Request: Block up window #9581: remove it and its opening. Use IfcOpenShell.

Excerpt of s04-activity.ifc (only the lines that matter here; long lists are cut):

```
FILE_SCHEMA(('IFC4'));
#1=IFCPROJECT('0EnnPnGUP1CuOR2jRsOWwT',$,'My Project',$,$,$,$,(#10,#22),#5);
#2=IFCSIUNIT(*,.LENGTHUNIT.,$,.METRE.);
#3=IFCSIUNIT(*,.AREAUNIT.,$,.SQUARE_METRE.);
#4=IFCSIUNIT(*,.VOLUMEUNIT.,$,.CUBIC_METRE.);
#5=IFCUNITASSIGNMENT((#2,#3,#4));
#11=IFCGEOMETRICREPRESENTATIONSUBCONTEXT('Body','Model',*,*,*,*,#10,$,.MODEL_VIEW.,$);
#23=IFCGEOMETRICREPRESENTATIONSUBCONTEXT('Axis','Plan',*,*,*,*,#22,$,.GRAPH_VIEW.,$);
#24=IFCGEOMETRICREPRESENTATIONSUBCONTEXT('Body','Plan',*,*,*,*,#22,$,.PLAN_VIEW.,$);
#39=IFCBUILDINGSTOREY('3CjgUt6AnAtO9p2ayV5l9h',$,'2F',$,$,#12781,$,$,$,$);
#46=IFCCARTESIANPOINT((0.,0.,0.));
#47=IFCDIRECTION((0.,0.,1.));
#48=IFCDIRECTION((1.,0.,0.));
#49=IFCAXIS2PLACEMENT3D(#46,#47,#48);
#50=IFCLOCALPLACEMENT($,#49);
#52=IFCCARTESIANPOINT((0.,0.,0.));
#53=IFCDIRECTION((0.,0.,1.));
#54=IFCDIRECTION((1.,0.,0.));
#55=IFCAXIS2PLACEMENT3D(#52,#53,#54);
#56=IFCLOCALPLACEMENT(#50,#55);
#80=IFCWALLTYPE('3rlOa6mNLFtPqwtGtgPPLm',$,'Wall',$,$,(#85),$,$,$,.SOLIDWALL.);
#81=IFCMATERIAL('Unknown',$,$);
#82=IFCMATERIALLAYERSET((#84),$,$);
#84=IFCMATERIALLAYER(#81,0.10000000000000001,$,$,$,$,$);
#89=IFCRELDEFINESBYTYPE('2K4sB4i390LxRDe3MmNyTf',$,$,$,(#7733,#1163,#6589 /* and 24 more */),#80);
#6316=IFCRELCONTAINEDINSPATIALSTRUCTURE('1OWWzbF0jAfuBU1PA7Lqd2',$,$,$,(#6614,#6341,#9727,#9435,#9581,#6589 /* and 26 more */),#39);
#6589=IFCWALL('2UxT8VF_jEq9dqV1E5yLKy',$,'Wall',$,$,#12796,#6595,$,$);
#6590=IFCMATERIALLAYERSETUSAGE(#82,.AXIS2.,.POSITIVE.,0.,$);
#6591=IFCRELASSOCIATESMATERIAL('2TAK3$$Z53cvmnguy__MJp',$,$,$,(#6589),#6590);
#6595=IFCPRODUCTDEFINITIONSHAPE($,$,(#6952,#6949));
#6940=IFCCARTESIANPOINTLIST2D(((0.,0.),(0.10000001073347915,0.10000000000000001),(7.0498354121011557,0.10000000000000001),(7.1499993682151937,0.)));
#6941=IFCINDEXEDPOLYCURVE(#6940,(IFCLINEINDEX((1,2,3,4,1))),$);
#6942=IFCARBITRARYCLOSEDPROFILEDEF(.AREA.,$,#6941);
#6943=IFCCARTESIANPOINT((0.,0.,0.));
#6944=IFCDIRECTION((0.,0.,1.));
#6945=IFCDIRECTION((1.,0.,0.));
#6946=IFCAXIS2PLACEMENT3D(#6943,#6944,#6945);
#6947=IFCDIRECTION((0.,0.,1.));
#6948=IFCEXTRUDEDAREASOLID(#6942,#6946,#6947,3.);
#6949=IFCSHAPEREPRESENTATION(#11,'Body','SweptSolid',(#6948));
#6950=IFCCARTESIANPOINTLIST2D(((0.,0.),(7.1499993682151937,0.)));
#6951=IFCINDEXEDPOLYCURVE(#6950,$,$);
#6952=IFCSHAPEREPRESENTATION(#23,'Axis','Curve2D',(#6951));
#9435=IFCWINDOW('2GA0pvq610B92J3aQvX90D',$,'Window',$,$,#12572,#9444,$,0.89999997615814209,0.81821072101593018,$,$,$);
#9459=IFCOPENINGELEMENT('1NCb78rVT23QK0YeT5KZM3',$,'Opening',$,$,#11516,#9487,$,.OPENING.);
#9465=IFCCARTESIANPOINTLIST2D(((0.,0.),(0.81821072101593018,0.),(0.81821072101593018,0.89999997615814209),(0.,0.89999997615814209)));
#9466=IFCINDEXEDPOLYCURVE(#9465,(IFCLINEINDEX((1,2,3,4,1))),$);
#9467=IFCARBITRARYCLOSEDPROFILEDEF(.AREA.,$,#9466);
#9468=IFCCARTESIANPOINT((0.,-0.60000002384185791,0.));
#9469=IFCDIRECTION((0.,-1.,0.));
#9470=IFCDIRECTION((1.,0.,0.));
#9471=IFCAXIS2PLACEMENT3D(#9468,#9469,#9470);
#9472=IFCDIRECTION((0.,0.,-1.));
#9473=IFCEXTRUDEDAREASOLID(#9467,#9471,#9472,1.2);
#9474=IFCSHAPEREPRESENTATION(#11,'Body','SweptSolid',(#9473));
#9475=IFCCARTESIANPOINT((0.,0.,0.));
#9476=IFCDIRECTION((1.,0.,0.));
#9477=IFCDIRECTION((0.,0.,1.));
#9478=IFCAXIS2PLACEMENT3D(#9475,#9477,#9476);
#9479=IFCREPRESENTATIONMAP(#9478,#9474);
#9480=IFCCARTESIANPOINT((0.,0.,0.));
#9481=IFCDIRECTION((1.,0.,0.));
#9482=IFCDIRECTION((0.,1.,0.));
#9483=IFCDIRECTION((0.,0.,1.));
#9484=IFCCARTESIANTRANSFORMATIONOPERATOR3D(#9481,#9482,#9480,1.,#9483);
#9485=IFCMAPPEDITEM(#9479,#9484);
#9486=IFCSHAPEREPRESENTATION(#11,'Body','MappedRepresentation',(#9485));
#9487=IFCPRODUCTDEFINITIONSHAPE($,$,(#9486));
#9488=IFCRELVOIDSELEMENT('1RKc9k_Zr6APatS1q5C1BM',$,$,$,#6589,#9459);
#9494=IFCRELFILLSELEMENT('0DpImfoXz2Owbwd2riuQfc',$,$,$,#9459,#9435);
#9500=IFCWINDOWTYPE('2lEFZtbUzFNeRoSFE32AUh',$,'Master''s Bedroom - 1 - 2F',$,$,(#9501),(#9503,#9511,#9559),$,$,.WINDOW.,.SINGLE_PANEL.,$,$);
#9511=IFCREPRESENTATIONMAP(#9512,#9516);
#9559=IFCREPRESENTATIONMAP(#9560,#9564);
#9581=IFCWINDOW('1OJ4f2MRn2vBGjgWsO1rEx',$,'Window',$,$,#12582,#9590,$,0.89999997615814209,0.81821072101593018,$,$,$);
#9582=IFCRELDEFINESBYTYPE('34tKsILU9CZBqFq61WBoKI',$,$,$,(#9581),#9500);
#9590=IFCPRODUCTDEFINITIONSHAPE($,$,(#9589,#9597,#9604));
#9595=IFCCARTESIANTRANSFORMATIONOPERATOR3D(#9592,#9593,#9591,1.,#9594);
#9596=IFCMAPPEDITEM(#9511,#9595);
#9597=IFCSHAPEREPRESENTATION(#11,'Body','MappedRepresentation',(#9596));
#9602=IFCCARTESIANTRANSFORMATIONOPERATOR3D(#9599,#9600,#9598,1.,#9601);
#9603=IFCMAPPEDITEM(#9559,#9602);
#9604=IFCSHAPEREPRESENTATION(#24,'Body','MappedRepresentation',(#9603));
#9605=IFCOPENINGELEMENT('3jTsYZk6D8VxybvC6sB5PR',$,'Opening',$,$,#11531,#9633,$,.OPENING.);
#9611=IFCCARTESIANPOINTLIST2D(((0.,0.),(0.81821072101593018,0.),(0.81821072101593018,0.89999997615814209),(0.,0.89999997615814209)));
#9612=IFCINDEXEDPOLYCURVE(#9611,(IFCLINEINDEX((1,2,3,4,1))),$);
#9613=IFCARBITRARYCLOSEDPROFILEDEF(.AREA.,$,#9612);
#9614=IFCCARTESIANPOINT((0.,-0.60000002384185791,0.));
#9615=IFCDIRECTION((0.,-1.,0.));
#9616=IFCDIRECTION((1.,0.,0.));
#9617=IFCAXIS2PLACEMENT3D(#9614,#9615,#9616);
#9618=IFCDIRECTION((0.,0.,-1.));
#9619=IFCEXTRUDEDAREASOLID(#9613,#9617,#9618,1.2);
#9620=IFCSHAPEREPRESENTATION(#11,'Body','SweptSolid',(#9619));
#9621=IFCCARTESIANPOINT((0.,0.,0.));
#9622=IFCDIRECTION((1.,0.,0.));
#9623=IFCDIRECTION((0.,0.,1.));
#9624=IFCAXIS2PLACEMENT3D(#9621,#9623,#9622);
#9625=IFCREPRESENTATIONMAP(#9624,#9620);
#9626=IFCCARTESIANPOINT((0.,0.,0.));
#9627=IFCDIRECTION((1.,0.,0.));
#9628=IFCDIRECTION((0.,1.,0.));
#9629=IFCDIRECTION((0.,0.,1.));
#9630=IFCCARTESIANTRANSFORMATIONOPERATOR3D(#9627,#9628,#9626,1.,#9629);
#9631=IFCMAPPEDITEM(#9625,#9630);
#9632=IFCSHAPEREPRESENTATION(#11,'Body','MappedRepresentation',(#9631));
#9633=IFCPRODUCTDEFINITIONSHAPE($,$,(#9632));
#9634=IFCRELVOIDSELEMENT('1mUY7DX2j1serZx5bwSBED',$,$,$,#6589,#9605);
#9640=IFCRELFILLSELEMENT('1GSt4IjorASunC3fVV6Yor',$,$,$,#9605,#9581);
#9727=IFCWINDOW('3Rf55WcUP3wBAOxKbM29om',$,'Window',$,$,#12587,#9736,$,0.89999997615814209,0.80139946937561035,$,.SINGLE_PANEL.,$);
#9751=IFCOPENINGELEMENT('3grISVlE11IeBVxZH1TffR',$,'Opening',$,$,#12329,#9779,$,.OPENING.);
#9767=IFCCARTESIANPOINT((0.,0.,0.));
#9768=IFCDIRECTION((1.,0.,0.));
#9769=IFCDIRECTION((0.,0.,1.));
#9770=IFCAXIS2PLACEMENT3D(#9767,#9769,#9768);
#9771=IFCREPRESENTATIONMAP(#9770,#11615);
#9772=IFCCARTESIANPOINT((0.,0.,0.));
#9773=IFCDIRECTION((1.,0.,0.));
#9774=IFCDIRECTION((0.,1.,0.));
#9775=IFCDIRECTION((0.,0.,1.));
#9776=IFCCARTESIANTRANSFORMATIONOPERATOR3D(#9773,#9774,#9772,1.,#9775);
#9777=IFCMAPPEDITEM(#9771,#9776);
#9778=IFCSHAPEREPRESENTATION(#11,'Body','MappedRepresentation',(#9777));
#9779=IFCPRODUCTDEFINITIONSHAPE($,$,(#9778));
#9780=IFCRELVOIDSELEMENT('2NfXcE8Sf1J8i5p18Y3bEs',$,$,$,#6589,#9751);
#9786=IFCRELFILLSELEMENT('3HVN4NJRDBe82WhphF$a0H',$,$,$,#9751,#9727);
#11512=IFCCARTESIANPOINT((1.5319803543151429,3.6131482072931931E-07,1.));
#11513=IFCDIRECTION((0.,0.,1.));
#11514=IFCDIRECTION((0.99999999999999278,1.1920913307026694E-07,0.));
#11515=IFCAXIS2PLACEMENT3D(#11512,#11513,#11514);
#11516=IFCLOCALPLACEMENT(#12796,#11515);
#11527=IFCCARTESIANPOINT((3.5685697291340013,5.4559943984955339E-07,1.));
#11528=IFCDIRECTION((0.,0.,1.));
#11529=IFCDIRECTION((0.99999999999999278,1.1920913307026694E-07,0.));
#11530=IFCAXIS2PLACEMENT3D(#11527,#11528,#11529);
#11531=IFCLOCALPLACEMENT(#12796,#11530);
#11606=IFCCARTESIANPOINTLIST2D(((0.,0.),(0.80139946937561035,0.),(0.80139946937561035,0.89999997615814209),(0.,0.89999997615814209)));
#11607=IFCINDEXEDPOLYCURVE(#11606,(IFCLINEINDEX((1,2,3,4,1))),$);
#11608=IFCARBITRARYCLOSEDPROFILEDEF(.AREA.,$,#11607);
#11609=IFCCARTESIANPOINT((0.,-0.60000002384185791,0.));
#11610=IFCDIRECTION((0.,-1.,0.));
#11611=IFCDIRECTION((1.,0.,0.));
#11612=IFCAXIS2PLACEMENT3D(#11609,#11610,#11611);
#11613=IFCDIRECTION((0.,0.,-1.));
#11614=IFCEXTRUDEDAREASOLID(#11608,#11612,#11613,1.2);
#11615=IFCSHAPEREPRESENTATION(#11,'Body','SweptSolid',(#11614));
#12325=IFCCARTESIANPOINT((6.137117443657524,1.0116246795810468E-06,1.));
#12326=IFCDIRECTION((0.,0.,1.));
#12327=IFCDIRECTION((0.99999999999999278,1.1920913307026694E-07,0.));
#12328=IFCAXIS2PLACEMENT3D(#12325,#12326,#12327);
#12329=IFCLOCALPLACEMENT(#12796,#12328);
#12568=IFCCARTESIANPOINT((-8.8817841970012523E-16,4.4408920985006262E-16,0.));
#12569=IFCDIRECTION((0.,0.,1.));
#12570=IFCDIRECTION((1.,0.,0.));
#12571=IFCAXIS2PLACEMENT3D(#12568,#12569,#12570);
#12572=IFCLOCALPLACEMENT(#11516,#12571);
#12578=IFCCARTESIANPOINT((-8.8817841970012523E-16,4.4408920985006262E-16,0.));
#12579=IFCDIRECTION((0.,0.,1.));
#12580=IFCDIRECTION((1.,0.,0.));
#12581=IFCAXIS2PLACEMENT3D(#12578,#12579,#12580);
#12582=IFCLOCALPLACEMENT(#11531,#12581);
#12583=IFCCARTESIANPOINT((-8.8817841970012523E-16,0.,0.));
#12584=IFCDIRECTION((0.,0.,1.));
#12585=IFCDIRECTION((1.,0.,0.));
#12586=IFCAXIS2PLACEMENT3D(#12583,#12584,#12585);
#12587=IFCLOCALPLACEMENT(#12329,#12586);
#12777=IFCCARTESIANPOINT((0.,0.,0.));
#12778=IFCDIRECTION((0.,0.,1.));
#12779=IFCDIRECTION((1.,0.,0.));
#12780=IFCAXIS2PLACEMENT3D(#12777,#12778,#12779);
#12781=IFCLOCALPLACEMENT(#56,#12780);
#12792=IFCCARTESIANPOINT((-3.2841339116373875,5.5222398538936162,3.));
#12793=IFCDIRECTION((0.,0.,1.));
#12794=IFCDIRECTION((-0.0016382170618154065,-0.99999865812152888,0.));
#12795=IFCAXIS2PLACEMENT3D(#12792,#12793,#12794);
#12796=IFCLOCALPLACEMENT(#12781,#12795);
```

```python
import ifcopenshell
import ifcopenshell.api.feature
import ifcopenshell.api.root
import ifcopenshell.geom
import ifcopenshell.util.shape

model = ifcopenshell.open("s04-activity.ifc")
settings = ifcopenshell.geom.settings()


def volume(element):
    """Net volume in cubic metres, openings subtracted."""
    shape = ifcopenshell.geom.create_shape(settings, element)
    return ifcopenshell.util.shape.get_volume(shape.geometry)


window = model.by_id(9581)
opening = window.FillsVoids[0].RelatingOpeningElement
wall = opening.VoidsElements[0].RelatingBuildingElement
before = volume(wall)

ifcopenshell.api.root.remove_product(model, product=window)
ifcopenshell.api.feature.remove_feature(model, feature=opening)

after = volume(wall)

print(f"wall volume {before:.3f} -> {after:.3f} m3")

model.write("s04-activity_rev.ifc")
```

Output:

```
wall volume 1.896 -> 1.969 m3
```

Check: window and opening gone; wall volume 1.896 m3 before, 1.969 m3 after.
